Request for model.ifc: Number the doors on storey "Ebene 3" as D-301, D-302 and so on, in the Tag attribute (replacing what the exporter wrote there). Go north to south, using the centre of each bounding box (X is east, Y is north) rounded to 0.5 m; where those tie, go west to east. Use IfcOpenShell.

First a look at what the model holds.

```python
import ifcopenshell
import ifcopenshell.util.element
import ifcopenshell.util.placement

model = ifcopenshell.open("model.ifc")
print(model.schema)
storey = next(s for s in model.by_type("IfcBuildingStorey") if s.Name == "Ebene 3")
doors = [e for e in ifcopenshell.util.element.get_decomposition(storey) if e.is_a("IfcDoor")]
for e in sorted(doors, key=lambda e: e.id()):
    origin = ifcopenshell.util.placement.get_local_placement(e.ObjectPlacement)[:3, 3]
    print(e.id(), e.Tag, e.Name, origin.round(2) + 0.0, sep=" | ")
```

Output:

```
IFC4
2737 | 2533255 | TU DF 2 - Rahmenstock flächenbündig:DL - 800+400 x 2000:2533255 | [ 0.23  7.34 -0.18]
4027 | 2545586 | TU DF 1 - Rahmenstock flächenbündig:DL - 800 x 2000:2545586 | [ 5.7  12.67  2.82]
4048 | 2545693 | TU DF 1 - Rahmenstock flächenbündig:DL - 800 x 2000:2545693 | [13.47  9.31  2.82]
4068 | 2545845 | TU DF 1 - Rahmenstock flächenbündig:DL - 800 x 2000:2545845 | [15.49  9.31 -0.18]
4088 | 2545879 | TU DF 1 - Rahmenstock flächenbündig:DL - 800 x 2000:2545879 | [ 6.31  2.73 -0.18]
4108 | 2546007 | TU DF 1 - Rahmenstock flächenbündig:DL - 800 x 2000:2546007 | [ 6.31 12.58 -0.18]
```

```python
import ifcopenshell
import ifcopenshell.geom
import ifcopenshell.util.element
import ifcopenshell.util.shape

model = ifcopenshell.open("model.ifc")
settings = ifcopenshell.geom.settings()
settings.set("use-world-coords", True)


def centre(element):
    shape = ifcopenshell.geom.create_shape(settings, element)
    return ifcopenshell.util.shape.get_bbox_centroid(shape.geometry)


storey = next(s for s in model.by_type("IfcBuildingStorey") if s.Name == "Ebene 3")
doors = [e for e in ifcopenshell.util.element.get_decomposition(storey) if e.is_a("IfcDoor")]

# Insertion points can sit at a corner or the storey origin, so sort by the geometry (in metres).
centres = {e: centre(e) for e in doors}
doors.sort(key=lambda e: (-round(centres[e][1] / 0.5), centres[e][0]))

for i, e in enumerate(doors, start=1):
    number = f"D-3{i:02d}"
    e.Tag = number
    print(e.id(), number)

model.write("model-out.ifc")
```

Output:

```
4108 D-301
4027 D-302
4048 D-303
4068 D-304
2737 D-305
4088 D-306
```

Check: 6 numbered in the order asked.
